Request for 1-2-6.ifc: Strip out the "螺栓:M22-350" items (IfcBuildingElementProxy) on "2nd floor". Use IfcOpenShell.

First a look at what the model holds.

```python
import ifcopenshell
import ifcopenshell.util.element

model = ifcopenshell.open("1-2-6.ifc")
print(model.schema)
storey = next(s for s in model.by_type("IfcBuildingStorey") if s.Name == "2nd floor")
proxies = [e for e in ifcopenshell.util.element.get_decomposition(storey) if e.is_a("IfcBuildingElementProxy")]
seen = {}
for e in proxies:
    element_type = ifcopenshell.util.element.get_type(e)
    name = element_type.Name if element_type not in (None, e) else None
    seen[name] = seen.get(name, 0) + 1
for name, count in sorted(seen.items(), key=str):
    print(count, "x", name)
```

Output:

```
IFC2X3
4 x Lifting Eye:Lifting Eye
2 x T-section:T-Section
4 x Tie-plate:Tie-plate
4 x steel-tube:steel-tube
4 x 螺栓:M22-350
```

```python
import ifcopenshell
import ifcopenshell.api.root
import ifcopenshell.util.element

model = ifcopenshell.open("1-2-6.ifc")

storey = next(s for s in model.by_type("IfcBuildingStorey") if s.Name == "2nd floor")
proxies = [e for e in ifcopenshell.util.element.get_decomposition(storey) if e.is_a("IfcBuildingElementProxy")]
targets = [e for e in proxies if (t := ifcopenshell.util.element.get_type(e)) not in (None, e) and t.Name == "螺栓:M22-350"]

for e in targets:
    ifcopenshell.api.root.remove_product(model, product=e)
print(len(targets), "removed")

model.write("1-2-6_rev.ifc")
```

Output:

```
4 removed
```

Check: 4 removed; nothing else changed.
